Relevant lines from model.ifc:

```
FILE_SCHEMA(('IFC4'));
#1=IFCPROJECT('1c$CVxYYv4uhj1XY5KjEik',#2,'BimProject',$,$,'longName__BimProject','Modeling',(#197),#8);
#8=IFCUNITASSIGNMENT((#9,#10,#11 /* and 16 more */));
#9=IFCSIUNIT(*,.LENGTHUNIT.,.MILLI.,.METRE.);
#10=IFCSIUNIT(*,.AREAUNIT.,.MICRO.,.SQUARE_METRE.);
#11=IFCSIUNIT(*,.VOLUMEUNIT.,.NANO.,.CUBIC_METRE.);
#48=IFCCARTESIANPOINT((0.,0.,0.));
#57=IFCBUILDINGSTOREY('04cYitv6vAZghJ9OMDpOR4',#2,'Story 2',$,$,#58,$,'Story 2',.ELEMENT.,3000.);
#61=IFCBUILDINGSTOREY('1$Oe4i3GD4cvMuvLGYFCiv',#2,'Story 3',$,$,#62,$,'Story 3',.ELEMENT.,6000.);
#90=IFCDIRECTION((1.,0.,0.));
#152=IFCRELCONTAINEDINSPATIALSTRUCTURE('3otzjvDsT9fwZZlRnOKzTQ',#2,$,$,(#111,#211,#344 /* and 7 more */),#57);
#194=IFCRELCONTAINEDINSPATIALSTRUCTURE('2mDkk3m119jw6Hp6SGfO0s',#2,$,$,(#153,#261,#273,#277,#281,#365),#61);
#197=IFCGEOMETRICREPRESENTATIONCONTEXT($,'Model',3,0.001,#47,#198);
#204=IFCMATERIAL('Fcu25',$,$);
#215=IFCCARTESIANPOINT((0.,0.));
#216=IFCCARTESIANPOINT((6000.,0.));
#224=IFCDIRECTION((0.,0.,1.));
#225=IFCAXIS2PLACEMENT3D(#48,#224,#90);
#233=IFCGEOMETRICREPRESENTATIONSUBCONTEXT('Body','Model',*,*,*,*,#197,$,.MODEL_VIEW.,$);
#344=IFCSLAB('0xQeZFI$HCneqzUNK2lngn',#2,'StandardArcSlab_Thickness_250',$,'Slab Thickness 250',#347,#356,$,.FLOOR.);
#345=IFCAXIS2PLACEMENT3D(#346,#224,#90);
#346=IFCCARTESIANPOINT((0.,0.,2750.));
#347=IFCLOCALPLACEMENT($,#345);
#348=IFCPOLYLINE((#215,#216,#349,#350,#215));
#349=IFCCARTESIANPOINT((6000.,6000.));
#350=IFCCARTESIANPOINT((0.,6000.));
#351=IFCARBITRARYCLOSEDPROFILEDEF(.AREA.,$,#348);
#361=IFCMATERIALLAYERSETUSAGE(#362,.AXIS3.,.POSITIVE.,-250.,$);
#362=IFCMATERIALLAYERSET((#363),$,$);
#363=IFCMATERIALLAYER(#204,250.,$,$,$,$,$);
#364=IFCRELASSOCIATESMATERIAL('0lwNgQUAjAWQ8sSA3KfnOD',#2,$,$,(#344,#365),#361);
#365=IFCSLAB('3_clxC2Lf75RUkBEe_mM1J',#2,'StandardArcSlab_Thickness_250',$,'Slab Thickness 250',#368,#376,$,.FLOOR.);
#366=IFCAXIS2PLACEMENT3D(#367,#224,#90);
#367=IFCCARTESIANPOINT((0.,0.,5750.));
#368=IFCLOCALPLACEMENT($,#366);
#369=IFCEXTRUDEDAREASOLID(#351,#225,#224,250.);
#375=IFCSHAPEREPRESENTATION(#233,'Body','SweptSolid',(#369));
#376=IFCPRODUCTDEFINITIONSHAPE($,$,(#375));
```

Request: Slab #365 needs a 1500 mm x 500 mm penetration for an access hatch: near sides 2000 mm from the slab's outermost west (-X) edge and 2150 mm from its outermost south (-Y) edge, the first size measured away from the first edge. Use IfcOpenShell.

```python
import numpy as np
import ifcopenshell
import ifcopenshell.api.feature
import ifcopenshell.api.geometry
import ifcopenshell.api.root
import ifcopenshell.geom
import ifcopenshell.util.placement
import ifcopenshell.util.representation
import ifcopenshell.util.shape
import ifcopenshell.util.unit

model = ifcopenshell.open("model.ifc")
unit_scale = ifcopenshell.util.unit.calculate_unit_scale(model)
settings = ifcopenshell.geom.settings()


def volume(element):
    """Net volume in cubic metres, openings subtracted."""
    shape = ifcopenshell.geom.create_shape(settings, element)
    return ifcopenshell.util.shape.get_volume(shape.geometry)


slab = model.by_guid("3_clxC2Lf75RUkBEe_mM1J")
before = volume(slab)

# Extent in the slab's own axes, in metres. The edges named are its -X and -Y sides.
slab_shape = ifcopenshell.geom.create_shape(settings, slab)
vertices = ifcopenshell.util.shape.get_vertices(slab_shape.geometry)
x_min, y_min, bottom = vertices.min(axis=0)
top = vertices[:, 2].max()

opening = ifcopenshell.api.root.create_entity(model, ifc_class="IfcOpeningElement", name="Access hatch opening", predefined_type="OPENING")
context = ifcopenshell.util.representation.get_context(model, "Model", "Body", "MODEL_VIEW")
width, depth = 1.5, 0.5
outline = [(0.0, 0.0), (width, 0.0), (width, depth), (0.0, depth), (0.0, 0.0)]
# Overshoot both faces by 50 mm so the cut is clean.
shape = ifcopenshell.api.geometry.add_slab_representation(
    model, context=context, depth=top - bottom + 0.1, polyline=outline
)
ifcopenshell.api.geometry.assign_representation(model, product=opening, representation=shape)

matrix = ifcopenshell.util.placement.get_local_placement(slab.ObjectPlacement)
matrix[:, 3] = matrix @ np.append(np.array([x_min + 2, y_min + 2.15, bottom - 0.05]) / unit_scale, 1.0)
ifcopenshell.api.geometry.edit_object_placement(model, product=opening, matrix=matrix, is_si=False)
ifcopenshell.api.feature.add_feature(model, feature=opening, element=slab)

after = volume(slab)

print(f"slab volume {before:.3f} -> {after:.3f} m3")

model.write("model_rev.ifc")
```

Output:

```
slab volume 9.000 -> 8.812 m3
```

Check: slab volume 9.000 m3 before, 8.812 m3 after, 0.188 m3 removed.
